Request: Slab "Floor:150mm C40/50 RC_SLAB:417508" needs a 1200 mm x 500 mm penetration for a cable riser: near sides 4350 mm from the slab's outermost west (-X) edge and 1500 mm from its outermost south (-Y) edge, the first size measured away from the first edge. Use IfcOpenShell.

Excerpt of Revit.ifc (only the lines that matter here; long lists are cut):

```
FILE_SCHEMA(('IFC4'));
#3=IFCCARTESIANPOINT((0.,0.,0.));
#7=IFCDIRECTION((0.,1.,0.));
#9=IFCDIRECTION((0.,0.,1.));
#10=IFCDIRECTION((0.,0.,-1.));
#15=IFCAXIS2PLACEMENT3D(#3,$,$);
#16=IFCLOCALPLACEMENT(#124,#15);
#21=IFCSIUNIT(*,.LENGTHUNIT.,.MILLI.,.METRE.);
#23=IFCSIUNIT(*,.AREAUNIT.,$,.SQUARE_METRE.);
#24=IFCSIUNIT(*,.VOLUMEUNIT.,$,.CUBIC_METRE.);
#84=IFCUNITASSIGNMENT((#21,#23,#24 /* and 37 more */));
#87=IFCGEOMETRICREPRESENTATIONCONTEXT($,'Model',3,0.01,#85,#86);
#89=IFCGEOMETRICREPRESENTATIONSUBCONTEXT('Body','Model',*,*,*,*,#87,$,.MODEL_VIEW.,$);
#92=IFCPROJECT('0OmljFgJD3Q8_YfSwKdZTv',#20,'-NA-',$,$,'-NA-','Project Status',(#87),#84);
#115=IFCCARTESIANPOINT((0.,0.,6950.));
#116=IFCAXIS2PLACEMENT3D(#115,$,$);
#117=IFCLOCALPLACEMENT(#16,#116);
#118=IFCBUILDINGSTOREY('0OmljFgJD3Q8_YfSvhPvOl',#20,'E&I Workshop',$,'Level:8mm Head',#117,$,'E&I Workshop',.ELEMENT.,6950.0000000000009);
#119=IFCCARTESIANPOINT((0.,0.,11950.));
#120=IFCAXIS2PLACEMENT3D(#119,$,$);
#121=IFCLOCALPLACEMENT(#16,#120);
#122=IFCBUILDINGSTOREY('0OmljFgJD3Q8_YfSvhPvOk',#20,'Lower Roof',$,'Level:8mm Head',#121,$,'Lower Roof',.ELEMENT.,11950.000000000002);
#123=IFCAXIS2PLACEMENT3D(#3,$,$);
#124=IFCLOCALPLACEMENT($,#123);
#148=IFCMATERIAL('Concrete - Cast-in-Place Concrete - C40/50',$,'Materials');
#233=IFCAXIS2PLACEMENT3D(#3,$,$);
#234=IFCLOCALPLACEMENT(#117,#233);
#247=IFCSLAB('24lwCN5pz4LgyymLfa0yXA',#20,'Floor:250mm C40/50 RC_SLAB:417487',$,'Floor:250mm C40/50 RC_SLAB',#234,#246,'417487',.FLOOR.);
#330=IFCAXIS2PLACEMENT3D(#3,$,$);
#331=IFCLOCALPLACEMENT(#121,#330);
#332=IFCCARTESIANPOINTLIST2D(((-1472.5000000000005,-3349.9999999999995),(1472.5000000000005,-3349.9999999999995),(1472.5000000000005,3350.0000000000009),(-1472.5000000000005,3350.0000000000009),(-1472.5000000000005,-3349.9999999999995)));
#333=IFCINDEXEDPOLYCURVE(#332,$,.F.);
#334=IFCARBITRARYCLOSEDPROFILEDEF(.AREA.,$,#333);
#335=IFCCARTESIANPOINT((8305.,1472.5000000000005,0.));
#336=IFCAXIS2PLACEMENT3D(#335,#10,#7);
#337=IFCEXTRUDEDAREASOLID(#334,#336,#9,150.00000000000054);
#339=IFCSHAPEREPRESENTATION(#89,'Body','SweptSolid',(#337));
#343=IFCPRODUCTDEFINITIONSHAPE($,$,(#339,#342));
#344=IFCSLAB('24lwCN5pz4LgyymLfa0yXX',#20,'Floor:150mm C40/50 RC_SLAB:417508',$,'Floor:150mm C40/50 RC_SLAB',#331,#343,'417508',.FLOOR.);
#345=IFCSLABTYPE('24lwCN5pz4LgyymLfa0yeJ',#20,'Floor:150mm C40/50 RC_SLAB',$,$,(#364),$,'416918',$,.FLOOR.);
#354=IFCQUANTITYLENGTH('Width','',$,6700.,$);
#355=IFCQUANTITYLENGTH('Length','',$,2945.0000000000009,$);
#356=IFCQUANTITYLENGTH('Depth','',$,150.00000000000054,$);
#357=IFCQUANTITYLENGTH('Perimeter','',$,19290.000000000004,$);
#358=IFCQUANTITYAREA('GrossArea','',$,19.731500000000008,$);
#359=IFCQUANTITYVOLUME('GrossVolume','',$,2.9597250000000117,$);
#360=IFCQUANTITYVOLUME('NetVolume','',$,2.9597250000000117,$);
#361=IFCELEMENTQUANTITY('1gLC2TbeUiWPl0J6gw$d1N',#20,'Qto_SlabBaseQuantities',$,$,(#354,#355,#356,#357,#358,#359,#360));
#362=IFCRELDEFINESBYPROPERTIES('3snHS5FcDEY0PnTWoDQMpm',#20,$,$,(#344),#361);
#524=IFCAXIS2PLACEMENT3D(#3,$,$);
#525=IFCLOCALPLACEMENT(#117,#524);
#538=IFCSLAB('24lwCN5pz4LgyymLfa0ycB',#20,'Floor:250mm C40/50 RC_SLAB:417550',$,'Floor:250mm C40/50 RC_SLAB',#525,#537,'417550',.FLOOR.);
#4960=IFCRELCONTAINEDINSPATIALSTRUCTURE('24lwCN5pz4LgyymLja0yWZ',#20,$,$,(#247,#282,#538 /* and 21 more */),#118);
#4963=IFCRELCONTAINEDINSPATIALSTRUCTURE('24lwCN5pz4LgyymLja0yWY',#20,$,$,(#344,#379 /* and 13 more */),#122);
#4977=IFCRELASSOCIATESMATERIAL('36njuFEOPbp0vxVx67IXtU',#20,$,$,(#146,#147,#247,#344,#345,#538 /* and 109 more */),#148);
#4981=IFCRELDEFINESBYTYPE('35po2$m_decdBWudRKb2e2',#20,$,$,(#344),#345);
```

```python
import numpy as np
import ifcopenshell
import ifcopenshell.api.feature
import ifcopenshell.api.geometry
import ifcopenshell.api.pset
import ifcopenshell.api.root
import ifcopenshell.geom
import ifcopenshell.util.element
import ifcopenshell.util.placement
import ifcopenshell.util.representation
import ifcopenshell.util.shape
import ifcopenshell.util.unit

model = ifcopenshell.open("Revit.ifc")
unit_scale = ifcopenshell.util.unit.calculate_unit_scale(model)
volume_scale = ifcopenshell.util.unit.calculate_unit_scale(model, "VOLUMEUNIT")
settings = ifcopenshell.geom.settings()


def volume(element):
    """Net volume in cubic metres, openings subtracted."""
    shape = ifcopenshell.geom.create_shape(settings, element)
    return ifcopenshell.util.shape.get_volume(shape.geometry)


slab = model.by_id(344)
before = volume(slab)

# Extent in the slab's own axes, in metres. The edges named are its -X and -Y sides.
slab_shape = ifcopenshell.geom.create_shape(settings, slab)
vertices = ifcopenshell.util.shape.get_vertices(slab_shape.geometry)
x_min, y_min, bottom = vertices.min(axis=0)
top = vertices[:, 2].max()

opening = ifcopenshell.api.root.create_entity(model, ifc_class="IfcOpeningElement", name="Cable riser opening", predefined_type="OPENING")
context = ifcopenshell.util.representation.get_context(model, "Model", "Body", "MODEL_VIEW")
width, depth = 1.2, 0.5
outline = [(0.0, 0.0), (width, 0.0), (width, depth), (0.0, depth), (0.0, 0.0)]
# Overshoot both faces by 50 mm so the cut is clean.
shape = ifcopenshell.api.geometry.add_slab_representation(
    model, context=context, depth=top - bottom + 0.1, polyline=outline
)
ifcopenshell.api.geometry.assign_representation(model, product=opening, representation=shape)

matrix = ifcopenshell.util.placement.get_local_placement(slab.ObjectPlacement)
matrix[:, 3] = matrix @ np.append(np.array([x_min + 4.35, y_min + 1.5, bottom - 0.05]) / unit_scale, 1.0)
ifcopenshell.api.geometry.edit_object_placement(model, product=opening, matrix=matrix, is_si=False)
ifcopenshell.api.feature.add_feature(model, feature=opening, element=slab)

after = volume(slab)

# Update the slab's stored quantities.
qto = model.by_id(ifcopenshell.util.element.get_pset(slab, "Qto_SlabBaseQuantities", should_inherit=False)["id"])
ifcopenshell.api.pset.edit_qto(model, qto=qto, properties={"NetVolume": after / volume_scale})

print(f"slab volume {before:.3f} -> {after:.3f} m3")

model.write("Revit_v2.ifc")
```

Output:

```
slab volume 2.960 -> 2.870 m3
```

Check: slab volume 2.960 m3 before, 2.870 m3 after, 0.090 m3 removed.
